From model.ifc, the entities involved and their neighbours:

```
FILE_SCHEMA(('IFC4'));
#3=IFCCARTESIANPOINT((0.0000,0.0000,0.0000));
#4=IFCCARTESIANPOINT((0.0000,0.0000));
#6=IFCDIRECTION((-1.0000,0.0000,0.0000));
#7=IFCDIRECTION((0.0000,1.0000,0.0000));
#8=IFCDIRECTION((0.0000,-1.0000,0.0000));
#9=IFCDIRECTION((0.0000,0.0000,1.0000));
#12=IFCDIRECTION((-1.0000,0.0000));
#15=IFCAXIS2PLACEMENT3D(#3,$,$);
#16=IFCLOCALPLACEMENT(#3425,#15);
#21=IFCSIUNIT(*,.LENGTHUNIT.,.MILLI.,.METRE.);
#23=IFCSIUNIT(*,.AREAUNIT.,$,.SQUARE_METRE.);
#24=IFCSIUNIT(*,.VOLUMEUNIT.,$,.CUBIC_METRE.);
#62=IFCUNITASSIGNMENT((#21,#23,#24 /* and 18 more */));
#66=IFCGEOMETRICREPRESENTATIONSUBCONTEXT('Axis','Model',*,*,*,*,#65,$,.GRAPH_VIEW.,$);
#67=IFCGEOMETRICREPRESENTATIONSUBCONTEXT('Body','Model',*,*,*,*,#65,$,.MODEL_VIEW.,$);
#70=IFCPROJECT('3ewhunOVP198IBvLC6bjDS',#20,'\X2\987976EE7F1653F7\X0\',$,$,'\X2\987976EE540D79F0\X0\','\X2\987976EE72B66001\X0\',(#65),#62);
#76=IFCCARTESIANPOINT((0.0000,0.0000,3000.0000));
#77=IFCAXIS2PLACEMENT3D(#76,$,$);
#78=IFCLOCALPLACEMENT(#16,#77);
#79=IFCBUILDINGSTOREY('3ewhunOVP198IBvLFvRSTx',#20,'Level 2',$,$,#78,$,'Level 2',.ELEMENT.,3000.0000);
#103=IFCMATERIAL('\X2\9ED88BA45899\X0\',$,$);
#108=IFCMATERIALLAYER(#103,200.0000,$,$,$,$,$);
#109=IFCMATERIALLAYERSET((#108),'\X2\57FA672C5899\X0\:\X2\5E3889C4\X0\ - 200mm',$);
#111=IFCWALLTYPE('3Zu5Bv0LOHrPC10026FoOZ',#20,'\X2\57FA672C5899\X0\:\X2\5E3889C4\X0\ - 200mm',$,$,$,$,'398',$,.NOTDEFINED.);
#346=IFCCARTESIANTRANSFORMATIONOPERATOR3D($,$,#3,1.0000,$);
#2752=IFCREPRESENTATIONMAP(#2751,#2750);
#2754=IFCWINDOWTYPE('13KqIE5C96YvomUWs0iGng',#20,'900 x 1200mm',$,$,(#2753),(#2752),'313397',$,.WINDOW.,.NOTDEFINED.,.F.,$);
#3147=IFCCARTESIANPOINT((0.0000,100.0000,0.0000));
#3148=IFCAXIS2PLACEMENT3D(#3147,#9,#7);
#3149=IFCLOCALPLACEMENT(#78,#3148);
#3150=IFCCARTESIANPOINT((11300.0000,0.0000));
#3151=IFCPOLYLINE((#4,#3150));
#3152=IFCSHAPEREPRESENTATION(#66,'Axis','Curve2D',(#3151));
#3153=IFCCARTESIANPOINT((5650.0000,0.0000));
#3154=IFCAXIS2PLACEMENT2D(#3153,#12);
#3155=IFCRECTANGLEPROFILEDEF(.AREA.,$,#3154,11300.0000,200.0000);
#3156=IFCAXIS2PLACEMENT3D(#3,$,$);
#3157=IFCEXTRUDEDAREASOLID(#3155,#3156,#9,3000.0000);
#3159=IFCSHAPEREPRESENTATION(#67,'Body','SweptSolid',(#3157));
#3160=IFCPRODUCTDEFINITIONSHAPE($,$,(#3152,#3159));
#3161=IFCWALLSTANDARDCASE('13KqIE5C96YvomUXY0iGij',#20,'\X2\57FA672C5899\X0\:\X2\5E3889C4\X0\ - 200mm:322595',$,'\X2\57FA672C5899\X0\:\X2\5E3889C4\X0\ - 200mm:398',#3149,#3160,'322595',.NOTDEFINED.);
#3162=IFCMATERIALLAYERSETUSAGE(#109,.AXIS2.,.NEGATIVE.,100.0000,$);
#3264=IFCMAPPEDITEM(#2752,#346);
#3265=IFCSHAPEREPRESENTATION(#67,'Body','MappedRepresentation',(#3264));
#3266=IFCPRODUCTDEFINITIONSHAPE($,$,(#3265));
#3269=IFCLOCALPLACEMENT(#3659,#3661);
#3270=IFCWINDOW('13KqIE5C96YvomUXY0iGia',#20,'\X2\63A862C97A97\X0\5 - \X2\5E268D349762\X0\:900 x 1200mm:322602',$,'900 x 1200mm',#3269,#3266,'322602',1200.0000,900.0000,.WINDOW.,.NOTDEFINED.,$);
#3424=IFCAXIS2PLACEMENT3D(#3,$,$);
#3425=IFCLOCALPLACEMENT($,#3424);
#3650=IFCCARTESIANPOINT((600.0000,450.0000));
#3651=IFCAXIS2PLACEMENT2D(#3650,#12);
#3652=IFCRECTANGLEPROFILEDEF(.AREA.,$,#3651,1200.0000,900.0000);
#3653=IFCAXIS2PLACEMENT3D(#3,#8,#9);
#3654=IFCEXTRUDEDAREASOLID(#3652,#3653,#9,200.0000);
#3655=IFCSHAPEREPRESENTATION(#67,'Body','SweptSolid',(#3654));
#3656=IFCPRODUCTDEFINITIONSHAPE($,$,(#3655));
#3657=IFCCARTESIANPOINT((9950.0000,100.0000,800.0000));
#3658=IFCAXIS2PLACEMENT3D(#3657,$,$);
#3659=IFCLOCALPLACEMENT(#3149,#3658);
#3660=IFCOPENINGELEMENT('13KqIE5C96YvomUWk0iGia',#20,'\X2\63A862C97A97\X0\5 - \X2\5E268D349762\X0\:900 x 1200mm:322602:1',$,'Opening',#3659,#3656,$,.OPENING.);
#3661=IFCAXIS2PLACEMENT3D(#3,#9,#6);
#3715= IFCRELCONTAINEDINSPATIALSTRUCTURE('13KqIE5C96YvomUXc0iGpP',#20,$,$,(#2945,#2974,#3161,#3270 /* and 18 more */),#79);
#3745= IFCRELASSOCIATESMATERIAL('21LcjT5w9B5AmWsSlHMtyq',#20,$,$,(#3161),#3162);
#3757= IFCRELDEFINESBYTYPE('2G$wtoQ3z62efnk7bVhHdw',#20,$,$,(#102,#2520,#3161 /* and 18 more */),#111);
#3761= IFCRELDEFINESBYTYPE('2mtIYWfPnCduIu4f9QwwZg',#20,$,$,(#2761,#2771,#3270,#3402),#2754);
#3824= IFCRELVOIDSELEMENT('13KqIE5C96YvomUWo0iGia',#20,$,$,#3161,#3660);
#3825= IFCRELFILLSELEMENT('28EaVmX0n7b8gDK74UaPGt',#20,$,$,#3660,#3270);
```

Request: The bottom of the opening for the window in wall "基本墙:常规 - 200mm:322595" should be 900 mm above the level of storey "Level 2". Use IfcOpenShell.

```python
import numpy as np
import ifcopenshell
import ifcopenshell.api.geometry
import ifcopenshell.geom
import ifcopenshell.util.element
import ifcopenshell.util.placement
import ifcopenshell.util.shape
import ifcopenshell.util.unit

model = ifcopenshell.open("model.ifc")
unit_scale = ifcopenshell.util.unit.calculate_unit_scale(model)

window = model.by_id(3270)
opening = window.FillsVoids[0].RelatingOpeningElement
storey = ifcopenshell.util.element.get_container(window, ifc_class="IfcBuildingStorey")
level = ifcopenshell.util.placement.get_local_placement(storey.ObjectPlacement)[2, 3]

# The opening's origin need not be at the sill, so measure its lowest point.
shape = ifcopenshell.geom.create_shape(ifcopenshell.geom.settings(), opening)
bottom = ifcopenshell.util.shape.get_shape_bottom_elevation(shape, shape.geometry) / unit_scale
dz = level + 900.0 - bottom

shift = np.array([0.0, 0.0, dz])
# The window is placed relative to its opening, so it follows when the opening moves.
matrix = ifcopenshell.util.placement.get_local_placement(opening.ObjectPlacement)
matrix[:3, 3] += shift
ifcopenshell.api.geometry.edit_object_placement(
    model, product=opening, matrix=matrix, is_si=False, should_transform_children=True
)

print(f"moved by {dz * unit_scale:+.3f} m")

model.write("model-out.ifc")
```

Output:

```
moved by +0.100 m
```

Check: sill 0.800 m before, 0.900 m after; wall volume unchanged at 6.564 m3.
